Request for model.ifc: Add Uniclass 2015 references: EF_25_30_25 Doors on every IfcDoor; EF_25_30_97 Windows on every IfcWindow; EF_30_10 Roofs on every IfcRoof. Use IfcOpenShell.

First a look at what the model holds.

```python
import ifcopenshell

model = ifcopenshell.open("model.ifc")
print(model.schema)
print("classifications:", [c.Name for c in model.by_type("IfcClassification")])
for ifc_class in ("IfcDoor", "IfcRoof", "IfcStair", "IfcWall", "IfcWindow"):
    print(ifc_class, len(model.by_type(ifc_class)))
```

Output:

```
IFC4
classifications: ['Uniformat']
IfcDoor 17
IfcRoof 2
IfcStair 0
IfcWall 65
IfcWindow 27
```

```python
import ifcopenshell
import ifcopenshell.api.classification

model = ifcopenshell.open("model.ifc")

system = ifcopenshell.api.classification.add_classification(model, classification="Uniclass 2015")

codes = {
    "IfcDoor": ("EF_25_30_25", "Doors"),
    "IfcWindow": ("EF_25_30_97", "Windows"),
    "IfcRoof": ("EF_30_10", "Roofs"),
}
for ifc_class, (code, name) in codes.items():
    products = model.by_type(ifc_class)
    ifcopenshell.api.classification.add_reference(
        model, products=products, classification=system, identification=code, name=name
    )
    print(code, len(products))

model.write("model_edited.ifc")
```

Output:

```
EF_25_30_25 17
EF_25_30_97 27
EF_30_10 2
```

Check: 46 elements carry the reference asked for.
